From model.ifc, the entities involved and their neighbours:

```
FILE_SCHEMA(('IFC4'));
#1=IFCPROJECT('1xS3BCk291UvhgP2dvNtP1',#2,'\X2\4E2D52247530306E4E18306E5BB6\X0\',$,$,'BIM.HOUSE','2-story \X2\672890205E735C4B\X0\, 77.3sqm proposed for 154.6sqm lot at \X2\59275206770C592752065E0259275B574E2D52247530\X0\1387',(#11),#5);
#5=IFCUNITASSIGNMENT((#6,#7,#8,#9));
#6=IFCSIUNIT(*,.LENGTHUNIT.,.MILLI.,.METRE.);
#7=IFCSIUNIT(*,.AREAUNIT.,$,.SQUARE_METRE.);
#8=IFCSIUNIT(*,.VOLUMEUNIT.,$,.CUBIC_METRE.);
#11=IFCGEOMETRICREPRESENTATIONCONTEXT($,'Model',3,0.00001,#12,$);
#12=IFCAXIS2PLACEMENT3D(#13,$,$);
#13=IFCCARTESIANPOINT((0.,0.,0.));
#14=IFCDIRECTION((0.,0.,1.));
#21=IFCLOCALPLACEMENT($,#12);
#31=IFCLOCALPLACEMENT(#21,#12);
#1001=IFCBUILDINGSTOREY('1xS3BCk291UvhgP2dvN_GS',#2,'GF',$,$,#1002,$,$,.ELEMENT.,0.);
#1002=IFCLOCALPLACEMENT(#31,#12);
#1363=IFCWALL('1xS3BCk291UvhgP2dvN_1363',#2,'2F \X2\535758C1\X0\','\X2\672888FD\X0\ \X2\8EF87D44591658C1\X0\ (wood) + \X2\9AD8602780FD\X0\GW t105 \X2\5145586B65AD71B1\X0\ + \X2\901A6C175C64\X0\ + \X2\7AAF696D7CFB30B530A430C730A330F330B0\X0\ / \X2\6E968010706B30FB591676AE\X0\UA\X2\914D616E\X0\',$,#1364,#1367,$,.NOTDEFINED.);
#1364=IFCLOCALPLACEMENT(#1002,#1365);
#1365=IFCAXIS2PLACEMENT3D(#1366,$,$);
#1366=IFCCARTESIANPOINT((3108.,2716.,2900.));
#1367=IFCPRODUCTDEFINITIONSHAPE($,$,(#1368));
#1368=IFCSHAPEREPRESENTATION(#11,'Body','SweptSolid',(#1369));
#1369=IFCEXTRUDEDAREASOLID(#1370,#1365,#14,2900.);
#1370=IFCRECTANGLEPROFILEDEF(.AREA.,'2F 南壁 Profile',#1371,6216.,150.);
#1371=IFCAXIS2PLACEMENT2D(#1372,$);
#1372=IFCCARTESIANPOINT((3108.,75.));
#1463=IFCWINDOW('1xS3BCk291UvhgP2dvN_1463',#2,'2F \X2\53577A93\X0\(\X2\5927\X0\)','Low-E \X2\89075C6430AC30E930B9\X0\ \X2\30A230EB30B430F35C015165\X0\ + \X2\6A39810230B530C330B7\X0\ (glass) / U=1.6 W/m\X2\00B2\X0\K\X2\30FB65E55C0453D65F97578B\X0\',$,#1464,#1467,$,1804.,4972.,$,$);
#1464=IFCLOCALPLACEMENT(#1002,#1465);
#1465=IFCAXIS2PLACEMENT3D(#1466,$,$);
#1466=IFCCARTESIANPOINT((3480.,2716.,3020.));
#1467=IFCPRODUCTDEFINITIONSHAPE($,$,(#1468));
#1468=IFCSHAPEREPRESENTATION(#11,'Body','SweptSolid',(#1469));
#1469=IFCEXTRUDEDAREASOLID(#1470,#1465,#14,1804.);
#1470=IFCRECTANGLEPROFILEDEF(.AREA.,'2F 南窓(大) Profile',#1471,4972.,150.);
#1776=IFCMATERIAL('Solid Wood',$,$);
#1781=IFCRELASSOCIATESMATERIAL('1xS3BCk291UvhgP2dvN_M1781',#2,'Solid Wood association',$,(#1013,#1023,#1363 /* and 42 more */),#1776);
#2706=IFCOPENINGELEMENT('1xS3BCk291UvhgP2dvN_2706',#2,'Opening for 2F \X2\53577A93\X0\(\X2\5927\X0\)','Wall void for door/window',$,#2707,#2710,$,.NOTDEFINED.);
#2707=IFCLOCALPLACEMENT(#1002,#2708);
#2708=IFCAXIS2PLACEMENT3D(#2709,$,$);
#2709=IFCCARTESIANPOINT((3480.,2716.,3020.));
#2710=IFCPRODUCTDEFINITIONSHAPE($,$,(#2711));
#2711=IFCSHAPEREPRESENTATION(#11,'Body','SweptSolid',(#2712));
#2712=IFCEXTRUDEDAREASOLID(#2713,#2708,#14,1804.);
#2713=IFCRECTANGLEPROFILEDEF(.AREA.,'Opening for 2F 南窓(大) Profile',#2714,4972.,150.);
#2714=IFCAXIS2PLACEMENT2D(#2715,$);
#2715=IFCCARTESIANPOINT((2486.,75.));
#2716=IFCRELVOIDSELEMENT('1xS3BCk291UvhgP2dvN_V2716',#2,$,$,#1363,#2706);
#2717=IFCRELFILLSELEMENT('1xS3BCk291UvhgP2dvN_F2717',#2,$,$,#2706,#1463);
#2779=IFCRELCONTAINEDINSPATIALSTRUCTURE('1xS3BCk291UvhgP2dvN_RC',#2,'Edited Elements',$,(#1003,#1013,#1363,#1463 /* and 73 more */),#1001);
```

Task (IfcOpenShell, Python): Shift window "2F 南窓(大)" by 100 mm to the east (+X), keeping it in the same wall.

```python
import ifcopenshell
import ifcopenshell.api.geometry
import ifcopenshell.util.placement

model = ifcopenshell.open("model.ifc")

window = model.by_guid("1xS3BCk291UvhgP2dvN_1463")
opening = window.FillsVoids[0].RelatingOpeningElement
wall = opening.VoidsElements[0].RelatingBuildingElement

wall_matrix = ifcopenshell.util.placement.get_local_placement(wall.ObjectPlacement)
shift = wall_matrix[:3, 0] * 100.0
before = ifcopenshell.util.placement.get_local_placement(window.ObjectPlacement)[:3, 3].copy()

# The window is not placed relative to its opening, so move both.
for product in (opening, window):
    matrix = ifcopenshell.util.placement.get_local_placement(product.ObjectPlacement)
    matrix[:3, 3] += shift
    ifcopenshell.api.geometry.edit_object_placement(model, product=product, matrix=matrix, is_si=False)

after = ifcopenshell.util.placement.get_local_placement(window.ObjectPlacement)[:3, 3]
print("window moved by", (after - before).round(3) + 0.0)

model.write("model_edited.ifc")
```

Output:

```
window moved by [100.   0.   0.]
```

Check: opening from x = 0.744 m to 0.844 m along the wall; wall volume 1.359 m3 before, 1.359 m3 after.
